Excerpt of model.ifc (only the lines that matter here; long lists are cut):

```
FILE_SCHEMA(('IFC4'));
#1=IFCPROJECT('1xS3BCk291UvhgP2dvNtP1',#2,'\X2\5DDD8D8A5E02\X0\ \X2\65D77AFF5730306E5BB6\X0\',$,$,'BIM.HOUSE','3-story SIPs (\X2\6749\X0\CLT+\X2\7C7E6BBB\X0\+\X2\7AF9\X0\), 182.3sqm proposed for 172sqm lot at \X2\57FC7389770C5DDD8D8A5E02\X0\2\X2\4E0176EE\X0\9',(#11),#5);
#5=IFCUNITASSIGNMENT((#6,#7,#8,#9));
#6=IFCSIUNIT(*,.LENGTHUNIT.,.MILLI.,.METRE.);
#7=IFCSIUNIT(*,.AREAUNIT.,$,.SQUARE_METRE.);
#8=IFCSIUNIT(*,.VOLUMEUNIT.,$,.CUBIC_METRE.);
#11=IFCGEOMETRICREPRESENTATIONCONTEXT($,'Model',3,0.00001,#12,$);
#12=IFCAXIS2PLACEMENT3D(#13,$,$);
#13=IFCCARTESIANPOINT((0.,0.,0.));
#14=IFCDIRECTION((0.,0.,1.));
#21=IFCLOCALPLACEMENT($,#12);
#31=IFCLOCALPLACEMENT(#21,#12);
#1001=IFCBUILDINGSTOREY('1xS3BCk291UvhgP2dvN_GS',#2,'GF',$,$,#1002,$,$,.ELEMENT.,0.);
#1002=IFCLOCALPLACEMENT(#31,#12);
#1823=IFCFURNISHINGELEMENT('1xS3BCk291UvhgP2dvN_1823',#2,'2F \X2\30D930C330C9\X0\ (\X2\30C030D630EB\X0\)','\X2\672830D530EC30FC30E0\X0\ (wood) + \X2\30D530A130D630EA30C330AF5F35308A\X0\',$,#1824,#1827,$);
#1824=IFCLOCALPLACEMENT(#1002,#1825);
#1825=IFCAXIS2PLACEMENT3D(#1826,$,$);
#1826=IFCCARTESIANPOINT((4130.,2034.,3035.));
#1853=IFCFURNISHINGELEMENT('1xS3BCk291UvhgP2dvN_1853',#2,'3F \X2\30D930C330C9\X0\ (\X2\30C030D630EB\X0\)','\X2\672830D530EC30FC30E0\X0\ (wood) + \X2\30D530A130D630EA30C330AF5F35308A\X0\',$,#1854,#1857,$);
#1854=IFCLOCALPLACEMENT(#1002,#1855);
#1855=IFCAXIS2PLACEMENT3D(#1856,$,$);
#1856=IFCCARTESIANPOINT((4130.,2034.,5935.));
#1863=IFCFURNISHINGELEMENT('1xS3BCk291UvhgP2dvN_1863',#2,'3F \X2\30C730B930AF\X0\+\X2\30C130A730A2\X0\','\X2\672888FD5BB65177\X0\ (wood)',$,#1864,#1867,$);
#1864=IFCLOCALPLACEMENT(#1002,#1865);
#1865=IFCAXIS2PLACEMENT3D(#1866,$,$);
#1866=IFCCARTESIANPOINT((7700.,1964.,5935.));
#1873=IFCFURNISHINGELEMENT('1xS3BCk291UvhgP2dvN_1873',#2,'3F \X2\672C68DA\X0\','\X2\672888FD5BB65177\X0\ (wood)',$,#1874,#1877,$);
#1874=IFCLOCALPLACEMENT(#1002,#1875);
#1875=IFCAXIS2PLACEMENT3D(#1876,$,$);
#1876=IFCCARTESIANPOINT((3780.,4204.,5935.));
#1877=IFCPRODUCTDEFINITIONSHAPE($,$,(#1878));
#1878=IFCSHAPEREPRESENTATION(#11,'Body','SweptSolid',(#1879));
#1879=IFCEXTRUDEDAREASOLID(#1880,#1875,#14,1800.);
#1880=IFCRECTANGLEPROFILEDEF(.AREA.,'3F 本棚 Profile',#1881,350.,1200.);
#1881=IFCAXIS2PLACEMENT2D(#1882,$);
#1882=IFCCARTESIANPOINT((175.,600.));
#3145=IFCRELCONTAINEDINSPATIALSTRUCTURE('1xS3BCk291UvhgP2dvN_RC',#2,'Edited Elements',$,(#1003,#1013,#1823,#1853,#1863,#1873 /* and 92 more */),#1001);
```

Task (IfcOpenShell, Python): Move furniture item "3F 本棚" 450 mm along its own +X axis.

```python
import ifcopenshell
import ifcopenshell.api.geometry
import ifcopenshell.util.placement
import ifcopenshell.util.unit

model = ifcopenshell.open("model.ifc")
unit_scale = ifcopenshell.util.unit.calculate_unit_scale(model)

item = model.by_id(1873)
matrix = ifcopenshell.util.placement.get_local_placement(item.ObjectPlacement)
matrix[:3, 3] += matrix[:3, 0] * 0.45 / unit_scale
ifcopenshell.api.geometry.edit_object_placement(model, product=item, matrix=matrix, is_si=False)

print(ifcopenshell.util.placement.get_local_placement(item.ObjectPlacement).round(3) + 0.0)

model.write("model-out.ifc")
```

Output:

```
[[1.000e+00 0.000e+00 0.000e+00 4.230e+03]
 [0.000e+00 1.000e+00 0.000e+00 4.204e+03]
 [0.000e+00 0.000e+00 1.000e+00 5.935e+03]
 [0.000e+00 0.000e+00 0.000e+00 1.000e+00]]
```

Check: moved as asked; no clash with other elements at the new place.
